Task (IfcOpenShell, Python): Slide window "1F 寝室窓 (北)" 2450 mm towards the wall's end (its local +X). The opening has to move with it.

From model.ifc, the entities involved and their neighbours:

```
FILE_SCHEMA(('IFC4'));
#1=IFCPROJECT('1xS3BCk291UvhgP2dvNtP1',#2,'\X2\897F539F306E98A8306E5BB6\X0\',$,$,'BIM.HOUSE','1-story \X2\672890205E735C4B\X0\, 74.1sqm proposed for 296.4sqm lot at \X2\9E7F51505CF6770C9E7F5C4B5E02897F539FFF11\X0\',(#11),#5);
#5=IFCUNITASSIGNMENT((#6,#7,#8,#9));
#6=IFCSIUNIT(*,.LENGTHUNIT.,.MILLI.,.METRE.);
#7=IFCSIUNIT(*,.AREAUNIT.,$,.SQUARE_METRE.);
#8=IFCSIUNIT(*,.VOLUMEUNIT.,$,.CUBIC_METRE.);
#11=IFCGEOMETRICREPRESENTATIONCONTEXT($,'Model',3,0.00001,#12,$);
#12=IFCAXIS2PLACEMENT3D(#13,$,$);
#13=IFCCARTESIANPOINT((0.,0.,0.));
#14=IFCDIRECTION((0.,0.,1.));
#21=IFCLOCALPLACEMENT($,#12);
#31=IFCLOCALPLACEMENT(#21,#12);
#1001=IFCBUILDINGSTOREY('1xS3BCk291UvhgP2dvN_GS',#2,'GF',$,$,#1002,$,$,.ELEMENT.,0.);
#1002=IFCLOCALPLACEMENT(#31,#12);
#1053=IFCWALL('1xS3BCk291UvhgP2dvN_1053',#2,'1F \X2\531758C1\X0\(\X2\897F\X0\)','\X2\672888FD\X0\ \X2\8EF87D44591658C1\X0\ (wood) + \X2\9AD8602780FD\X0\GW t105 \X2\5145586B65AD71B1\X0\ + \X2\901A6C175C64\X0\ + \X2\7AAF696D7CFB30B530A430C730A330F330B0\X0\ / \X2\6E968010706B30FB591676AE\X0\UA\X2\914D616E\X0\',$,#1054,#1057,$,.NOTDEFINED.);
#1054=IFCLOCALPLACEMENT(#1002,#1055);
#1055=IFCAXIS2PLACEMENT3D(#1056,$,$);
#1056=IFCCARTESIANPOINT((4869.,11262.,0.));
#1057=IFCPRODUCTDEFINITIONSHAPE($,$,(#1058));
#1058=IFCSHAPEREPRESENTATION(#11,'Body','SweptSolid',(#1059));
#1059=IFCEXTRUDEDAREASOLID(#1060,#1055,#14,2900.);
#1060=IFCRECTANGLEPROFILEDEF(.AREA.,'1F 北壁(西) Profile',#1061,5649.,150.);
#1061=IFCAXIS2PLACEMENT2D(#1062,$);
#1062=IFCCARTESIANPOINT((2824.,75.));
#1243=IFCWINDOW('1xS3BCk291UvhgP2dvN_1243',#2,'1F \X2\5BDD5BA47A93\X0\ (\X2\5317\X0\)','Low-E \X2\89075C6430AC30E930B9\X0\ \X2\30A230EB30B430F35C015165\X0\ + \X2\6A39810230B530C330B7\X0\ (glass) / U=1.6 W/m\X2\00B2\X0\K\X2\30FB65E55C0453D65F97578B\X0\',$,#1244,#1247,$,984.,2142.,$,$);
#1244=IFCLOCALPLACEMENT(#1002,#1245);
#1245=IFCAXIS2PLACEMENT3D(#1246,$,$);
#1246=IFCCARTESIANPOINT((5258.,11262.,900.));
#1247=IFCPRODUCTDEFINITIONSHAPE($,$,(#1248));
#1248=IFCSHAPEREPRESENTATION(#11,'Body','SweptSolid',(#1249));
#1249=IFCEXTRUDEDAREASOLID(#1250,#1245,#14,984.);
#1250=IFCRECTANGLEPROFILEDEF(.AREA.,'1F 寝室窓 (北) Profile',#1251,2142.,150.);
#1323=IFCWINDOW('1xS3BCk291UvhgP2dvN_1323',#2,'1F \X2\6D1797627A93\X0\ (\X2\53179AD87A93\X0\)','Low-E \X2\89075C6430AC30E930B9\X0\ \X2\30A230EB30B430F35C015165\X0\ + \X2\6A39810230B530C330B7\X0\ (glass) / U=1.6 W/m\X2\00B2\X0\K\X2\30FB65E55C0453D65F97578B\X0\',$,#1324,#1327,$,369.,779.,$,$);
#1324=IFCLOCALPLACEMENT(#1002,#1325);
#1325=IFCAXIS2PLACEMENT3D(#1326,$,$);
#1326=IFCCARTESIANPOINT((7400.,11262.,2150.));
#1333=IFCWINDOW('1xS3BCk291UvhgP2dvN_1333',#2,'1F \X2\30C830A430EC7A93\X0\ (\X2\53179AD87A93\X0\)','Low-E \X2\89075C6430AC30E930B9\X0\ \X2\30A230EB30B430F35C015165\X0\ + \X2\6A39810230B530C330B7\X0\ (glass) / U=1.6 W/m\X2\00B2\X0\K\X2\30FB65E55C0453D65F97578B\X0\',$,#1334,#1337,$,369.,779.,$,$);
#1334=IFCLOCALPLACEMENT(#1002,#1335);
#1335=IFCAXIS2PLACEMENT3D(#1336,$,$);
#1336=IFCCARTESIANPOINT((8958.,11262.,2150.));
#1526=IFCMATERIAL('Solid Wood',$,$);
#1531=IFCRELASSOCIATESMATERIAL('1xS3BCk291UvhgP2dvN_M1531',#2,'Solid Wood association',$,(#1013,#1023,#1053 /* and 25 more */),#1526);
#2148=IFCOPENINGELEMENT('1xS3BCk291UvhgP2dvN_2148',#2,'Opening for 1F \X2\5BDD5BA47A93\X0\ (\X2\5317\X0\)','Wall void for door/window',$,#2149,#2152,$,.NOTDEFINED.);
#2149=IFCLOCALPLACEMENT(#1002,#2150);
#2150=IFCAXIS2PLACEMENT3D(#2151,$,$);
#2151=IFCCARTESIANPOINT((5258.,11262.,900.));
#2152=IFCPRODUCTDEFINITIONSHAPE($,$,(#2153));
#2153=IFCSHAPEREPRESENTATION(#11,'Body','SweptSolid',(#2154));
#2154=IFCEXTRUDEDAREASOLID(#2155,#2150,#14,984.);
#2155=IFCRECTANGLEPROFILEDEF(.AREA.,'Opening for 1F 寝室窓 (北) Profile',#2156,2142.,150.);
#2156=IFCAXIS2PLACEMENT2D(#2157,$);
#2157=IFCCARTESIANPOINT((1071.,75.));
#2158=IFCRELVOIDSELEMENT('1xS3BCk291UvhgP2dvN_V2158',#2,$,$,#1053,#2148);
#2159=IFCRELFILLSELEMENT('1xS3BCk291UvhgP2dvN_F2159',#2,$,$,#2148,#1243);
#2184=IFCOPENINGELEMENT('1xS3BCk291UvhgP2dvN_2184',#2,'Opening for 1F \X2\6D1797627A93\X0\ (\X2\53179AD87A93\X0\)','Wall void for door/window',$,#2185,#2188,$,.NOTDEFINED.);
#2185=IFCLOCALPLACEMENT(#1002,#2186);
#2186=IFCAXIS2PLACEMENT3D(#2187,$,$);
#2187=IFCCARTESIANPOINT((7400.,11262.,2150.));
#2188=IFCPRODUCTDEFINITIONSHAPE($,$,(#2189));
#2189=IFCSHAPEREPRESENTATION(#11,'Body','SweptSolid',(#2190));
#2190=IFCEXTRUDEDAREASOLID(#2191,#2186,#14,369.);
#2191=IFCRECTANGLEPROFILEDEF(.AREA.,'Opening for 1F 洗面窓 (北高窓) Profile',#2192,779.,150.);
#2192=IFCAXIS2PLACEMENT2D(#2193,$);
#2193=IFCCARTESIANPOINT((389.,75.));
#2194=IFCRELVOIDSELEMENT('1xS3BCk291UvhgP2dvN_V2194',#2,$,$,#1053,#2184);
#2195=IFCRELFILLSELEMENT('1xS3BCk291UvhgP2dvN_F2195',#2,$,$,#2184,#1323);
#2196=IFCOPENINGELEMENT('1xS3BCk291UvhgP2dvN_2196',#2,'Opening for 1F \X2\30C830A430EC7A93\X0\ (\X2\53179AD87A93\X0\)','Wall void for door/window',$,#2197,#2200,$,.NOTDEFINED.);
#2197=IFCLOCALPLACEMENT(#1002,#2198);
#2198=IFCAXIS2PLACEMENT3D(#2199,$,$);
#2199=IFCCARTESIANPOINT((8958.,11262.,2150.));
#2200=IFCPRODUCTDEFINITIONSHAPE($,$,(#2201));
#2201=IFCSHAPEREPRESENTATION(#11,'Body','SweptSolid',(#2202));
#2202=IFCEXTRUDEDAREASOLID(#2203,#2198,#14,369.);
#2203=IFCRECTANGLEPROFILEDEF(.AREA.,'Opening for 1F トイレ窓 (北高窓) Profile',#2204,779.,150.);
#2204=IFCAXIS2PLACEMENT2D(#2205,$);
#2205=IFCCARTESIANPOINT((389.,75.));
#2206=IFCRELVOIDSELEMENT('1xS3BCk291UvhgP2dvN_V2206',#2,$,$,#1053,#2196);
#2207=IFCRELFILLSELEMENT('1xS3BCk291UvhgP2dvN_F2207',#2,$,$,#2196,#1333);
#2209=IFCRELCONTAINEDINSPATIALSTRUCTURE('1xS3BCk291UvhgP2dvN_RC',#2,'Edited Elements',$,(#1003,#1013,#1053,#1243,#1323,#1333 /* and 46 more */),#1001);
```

```python
import ifcopenshell
import ifcopenshell.api.geometry
import ifcopenshell.util.placement
import ifcopenshell.util.unit

model = ifcopenshell.open("model.ifc")
unit_scale = ifcopenshell.util.unit.calculate_unit_scale(model)

window = model.by_guid("1xS3BCk291UvhgP2dvN_1243")
opening = window.FillsVoids[0].RelatingOpeningElement
wall = opening.VoidsElements[0].RelatingBuildingElement

wall_matrix = ifcopenshell.util.placement.get_local_placement(wall.ObjectPlacement)
shift = wall_matrix[:3, 0] * 2.45 / unit_scale
before = ifcopenshell.util.placement.get_local_placement(window.ObjectPlacement)[:3, 3].copy()

# The window is not placed relative to its opening, so move both.
for product in (opening, window):
    matrix = ifcopenshell.util.placement.get_local_placement(product.ObjectPlacement)
    matrix[:3, 3] += shift
    ifcopenshell.api.geometry.edit_object_placement(model, product=product, matrix=matrix, is_si=False)

after = ifcopenshell.util.placement.get_local_placement(window.ObjectPlacement)[:3, 3]
print("window moved by", (after - before).round(3) + 0.0)

model.write("model_rev.ifc")
```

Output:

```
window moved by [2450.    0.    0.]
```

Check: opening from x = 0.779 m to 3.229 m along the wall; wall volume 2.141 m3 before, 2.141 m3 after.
